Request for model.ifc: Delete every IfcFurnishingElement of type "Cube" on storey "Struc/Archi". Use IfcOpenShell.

First a look at what the model holds.

```python
import ifcopenshell
import ifcopenshell.util.element

model = ifcopenshell.open("model.ifc")
print(model.schema)
storey = next(s for s in model.by_type("IfcBuildingStorey") if s.Name == "Struc/Archi")
furniture = [e for e in ifcopenshell.util.element.get_decomposition(storey) if e.is_a("IfcFurnishingElement")]
seen = {}
for e in furniture:
    element_type = ifcopenshell.util.element.get_type(e)
    name = element_type.Name if element_type not in (None, e) else None
    seen[name] = seen.get(name, 0) + 1
for name, count in sorted(seen.items(), key=str):
    print(count, "x", name)
```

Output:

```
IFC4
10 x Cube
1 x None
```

```python
import ifcopenshell
import ifcopenshell.api.root
import ifcopenshell.util.element

model = ifcopenshell.open("model.ifc")

storey = next(s for s in model.by_type("IfcBuildingStorey") if s.Name == "Struc/Archi")
furniture = [e for e in ifcopenshell.util.element.get_decomposition(storey) if e.is_a("IfcFurnishingElement")]
targets = [e for e in furniture if (t := ifcopenshell.util.element.get_type(e)) not in (None, e) and t.Name == "Cube"]

for e in targets:
    ifcopenshell.api.root.remove_product(model, product=e)
print(len(targets), "removed")

model.write("model_updated.ifc")
```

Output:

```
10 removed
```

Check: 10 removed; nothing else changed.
